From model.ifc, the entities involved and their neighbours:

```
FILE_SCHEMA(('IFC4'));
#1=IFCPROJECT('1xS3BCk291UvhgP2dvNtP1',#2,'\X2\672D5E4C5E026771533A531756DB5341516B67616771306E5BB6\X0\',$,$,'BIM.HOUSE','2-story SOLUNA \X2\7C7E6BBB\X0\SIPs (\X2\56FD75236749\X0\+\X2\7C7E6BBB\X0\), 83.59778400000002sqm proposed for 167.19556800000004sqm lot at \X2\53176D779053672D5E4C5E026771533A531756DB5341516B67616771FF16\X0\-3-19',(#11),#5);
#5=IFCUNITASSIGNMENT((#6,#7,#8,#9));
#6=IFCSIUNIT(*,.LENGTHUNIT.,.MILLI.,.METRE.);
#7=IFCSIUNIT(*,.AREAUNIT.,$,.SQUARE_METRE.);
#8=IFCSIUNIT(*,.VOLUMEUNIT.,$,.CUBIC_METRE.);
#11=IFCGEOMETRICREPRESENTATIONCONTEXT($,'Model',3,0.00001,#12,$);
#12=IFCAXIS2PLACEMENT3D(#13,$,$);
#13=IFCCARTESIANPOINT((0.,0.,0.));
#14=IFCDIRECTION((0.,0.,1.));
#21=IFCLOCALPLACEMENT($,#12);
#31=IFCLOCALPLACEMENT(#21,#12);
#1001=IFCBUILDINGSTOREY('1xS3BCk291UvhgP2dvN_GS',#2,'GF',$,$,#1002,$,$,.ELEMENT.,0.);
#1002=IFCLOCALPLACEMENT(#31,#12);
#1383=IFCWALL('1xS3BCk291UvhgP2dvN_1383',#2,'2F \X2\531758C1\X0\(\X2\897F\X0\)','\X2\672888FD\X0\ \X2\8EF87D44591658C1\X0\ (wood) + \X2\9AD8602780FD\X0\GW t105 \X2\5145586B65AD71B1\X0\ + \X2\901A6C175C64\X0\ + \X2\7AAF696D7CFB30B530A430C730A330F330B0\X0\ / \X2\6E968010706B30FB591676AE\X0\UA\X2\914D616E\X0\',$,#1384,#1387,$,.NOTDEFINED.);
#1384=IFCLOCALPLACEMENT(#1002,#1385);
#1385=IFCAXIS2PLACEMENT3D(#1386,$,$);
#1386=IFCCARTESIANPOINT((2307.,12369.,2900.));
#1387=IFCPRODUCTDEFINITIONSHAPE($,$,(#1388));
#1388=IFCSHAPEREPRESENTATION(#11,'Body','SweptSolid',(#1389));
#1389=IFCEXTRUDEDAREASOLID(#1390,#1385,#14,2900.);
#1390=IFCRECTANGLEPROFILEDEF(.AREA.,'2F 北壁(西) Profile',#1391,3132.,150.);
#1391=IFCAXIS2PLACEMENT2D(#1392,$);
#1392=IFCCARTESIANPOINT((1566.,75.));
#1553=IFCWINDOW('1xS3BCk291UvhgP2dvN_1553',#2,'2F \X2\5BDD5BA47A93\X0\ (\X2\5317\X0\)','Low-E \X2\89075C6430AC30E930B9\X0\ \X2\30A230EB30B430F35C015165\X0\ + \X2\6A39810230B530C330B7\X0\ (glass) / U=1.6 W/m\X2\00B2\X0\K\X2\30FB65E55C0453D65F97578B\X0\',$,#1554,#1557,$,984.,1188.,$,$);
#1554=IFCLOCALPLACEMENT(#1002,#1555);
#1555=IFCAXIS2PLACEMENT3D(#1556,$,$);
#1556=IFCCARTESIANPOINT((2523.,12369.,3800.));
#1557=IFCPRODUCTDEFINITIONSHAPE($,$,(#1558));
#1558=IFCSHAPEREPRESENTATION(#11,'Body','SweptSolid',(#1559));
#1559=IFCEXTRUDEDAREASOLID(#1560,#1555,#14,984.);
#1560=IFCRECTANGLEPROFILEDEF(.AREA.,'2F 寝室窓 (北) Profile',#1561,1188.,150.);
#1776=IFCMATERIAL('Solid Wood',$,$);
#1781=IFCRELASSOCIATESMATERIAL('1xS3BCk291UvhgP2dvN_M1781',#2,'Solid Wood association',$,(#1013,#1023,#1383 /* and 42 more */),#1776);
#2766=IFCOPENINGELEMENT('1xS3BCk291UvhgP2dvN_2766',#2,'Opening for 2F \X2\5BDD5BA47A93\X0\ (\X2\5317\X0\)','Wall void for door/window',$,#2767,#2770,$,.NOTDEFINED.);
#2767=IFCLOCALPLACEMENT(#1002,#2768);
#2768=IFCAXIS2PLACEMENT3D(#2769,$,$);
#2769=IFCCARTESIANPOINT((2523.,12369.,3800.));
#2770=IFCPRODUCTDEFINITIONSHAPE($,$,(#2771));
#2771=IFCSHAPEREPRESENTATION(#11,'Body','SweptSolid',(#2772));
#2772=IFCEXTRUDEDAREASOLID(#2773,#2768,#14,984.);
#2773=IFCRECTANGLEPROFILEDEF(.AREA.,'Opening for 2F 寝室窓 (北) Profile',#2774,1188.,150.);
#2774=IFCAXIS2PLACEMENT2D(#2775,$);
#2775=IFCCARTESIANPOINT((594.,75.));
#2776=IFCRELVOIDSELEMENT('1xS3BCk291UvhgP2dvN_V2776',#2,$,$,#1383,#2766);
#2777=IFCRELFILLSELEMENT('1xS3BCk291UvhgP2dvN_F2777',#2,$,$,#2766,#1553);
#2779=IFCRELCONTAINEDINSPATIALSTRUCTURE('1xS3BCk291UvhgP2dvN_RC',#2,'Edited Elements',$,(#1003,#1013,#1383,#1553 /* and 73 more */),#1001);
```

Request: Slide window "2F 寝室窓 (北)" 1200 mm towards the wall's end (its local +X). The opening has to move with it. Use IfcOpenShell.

```python
import ifcopenshell
import ifcopenshell.api.geometry
import ifcopenshell.util.placement

model = ifcopenshell.open("model.ifc")

window = model.by_guid("1xS3BCk291UvhgP2dvN_1553")
opening = window.FillsVoids[0].RelatingOpeningElement
wall = opening.VoidsElements[0].RelatingBuildingElement

wall_matrix = ifcopenshell.util.placement.get_local_placement(wall.ObjectPlacement)
shift = wall_matrix[:3, 0] * 1200.0
before = ifcopenshell.util.placement.get_local_placement(window.ObjectPlacement)[:3, 3].copy()

# The window is not placed relative to its opening, so move both.
for product in (opening, window):
    matrix = ifcopenshell.util.placement.get_local_placement(product.ObjectPlacement)
    matrix[:3, 3] += shift
    ifcopenshell.api.geometry.edit_object_placement(model, product=product, matrix=matrix, is_si=False)

after = ifcopenshell.util.placement.get_local_placement(window.ObjectPlacement)[:3, 3]
print("window moved by", (after - before).round(3) + 0.0)

model.write("model_v2.ifc")
```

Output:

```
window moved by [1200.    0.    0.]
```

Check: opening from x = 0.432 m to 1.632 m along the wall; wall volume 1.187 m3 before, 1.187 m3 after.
